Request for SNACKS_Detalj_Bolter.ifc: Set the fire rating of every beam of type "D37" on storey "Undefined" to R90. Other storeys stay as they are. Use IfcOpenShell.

First a look at what the model holds.

```python
import ifcopenshell
import ifcopenshell.util.element

model = ifcopenshell.open("SNACKS_Detalj_Bolter.ifc")
print(model.schema)
storey = next(s for s in model.by_type("IfcBuildingStorey") if s.Name == "Undefined")
beams = [e for e in ifcopenshell.util.element.get_decomposition(storey) if e.is_a("IfcBeam")]
seen = {}
for e in beams:
    element_type = ifcopenshell.util.element.get_type(e)
    key = (element_type.Name if element_type != e and element_type else None, ifcopenshell.util.element.get_pset(e, "Pset_BeamCommon", "FireRating"))
    seen[key] = seen.get(key, 0) + 1
for (name, value), count in sorted(seen.items(), key=str):
    print(count, "x", name, "|", value)
```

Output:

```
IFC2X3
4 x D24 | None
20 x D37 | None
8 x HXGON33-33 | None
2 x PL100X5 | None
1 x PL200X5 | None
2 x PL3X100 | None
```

```python
import ifcopenshell
import ifcopenshell.api.pset
import ifcopenshell.util.element

model = ifcopenshell.open("SNACKS_Detalj_Bolter.ifc")

storey = next(s for s in model.by_type("IfcBuildingStorey") if s.Name == "Undefined")
beams = [e for e in ifcopenshell.util.element.get_decomposition(storey) if e.is_a("IfcBeam")]

count = 0
for e in beams:
    element_type = ifcopenshell.util.element.get_type(e)
    if element_type in (None, e) or element_type.Name != "D37":
        continue
    # add_pset returns the element's existing set when there is one.
    pset = ifcopenshell.api.pset.add_pset(model, product=e, name="Pset_BeamCommon")
    ifcopenshell.api.pset.edit_pset(model, pset=pset, properties={"FireRating": "R90"})
    count += 1

print(count, "beams updated")

model.write("SNACKS_Detalj_Bolter_updated.ifc")
```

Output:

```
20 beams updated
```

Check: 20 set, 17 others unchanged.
